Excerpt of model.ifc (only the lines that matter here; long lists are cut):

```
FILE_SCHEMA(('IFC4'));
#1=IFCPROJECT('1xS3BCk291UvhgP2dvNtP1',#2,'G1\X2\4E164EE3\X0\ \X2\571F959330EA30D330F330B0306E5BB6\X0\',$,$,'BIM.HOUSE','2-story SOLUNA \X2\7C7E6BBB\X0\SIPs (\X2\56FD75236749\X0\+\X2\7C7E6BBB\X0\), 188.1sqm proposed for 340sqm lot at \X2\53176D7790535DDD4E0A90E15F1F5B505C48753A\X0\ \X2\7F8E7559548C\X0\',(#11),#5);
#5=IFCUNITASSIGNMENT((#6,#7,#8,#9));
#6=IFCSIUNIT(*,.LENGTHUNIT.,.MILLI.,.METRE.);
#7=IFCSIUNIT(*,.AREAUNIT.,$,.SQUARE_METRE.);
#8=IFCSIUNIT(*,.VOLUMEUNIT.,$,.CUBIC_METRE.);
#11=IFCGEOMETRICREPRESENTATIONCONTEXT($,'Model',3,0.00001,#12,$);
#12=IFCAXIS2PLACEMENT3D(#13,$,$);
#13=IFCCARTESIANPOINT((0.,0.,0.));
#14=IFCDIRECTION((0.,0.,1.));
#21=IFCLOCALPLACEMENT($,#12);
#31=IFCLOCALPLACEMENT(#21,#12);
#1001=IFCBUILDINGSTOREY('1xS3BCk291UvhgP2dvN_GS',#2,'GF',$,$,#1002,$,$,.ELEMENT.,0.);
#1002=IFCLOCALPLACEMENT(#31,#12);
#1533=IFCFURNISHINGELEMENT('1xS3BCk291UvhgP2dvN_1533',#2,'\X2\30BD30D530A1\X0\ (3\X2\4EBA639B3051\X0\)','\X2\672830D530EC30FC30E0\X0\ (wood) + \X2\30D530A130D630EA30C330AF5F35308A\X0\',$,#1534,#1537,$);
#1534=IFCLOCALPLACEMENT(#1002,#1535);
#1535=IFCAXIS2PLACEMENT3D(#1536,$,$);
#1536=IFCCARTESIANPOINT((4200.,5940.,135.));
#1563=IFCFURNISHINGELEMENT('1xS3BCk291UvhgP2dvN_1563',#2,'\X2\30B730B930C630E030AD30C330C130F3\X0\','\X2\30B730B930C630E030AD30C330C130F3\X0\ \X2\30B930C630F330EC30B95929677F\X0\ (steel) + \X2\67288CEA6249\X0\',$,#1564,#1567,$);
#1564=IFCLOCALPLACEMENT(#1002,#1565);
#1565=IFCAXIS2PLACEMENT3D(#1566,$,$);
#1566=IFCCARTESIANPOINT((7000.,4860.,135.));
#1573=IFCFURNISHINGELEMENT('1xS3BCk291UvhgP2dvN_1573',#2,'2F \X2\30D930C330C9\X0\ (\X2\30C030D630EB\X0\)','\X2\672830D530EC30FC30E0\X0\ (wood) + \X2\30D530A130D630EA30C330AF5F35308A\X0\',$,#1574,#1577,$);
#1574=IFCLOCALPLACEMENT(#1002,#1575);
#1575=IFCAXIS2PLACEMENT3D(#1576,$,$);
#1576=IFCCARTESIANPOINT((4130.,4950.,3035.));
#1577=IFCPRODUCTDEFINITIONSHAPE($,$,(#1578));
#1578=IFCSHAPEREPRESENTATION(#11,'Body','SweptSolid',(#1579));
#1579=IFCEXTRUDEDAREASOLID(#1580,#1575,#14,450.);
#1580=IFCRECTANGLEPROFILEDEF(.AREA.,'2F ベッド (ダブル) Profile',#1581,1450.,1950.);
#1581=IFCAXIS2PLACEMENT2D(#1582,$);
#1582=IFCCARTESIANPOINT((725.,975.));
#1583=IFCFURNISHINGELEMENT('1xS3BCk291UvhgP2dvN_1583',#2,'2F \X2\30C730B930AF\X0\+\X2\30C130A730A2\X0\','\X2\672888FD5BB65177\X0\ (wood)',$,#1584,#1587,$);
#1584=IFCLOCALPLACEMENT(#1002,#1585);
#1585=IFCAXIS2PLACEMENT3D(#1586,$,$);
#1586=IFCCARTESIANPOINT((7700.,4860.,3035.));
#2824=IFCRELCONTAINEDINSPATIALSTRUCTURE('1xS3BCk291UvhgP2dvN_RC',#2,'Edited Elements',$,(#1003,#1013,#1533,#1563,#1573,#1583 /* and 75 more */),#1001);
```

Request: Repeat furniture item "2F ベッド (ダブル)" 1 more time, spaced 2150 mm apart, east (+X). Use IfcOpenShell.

```python
import numpy as np
import ifcopenshell
import ifcopenshell.api.geometry
import ifcopenshell.api.root
import ifcopenshell.util.element
import ifcopenshell.util.placement

model = ifcopenshell.open("model.ifc")


def reuse_history(source, copy):
    """copy_class also copies each property set's owner history, people and application; keep the originals."""
    for rel in copy.IsDefinedBy:
        if rel.is_a("IfcRelDefinesByProperties") and (history := rel.RelatingPropertyDefinition.OwnerHistory):
            rel.RelatingPropertyDefinition.OwnerHistory = source.OwnerHistory
            ifcopenshell.util.element.remove_deep2(model, history)


source = model.by_id(1573)
base = ifcopenshell.util.placement.get_local_placement(source.ObjectPlacement)
step = np.array([1.0, 0.0, 0.0]) * 2150.0

for i in range(1, 2):
    copy = ifcopenshell.api.root.copy_class(model, product=source)
    copy.Representation = ifcopenshell.util.element.copy_deep(
        model, source.Representation, exclude=["IfcGeometricRepresentationContext", "IfcRepresentationMap"]
    )
    reuse_history(source, copy)
    matrix = base.copy()
    matrix[:3, 3] += i * step
    print("added at", matrix[:3, 3].round(3) + 0.0)
    ifcopenshell.api.geometry.edit_object_placement(model, product=copy, matrix=matrix, is_si=False)

model.write("model_rev.ifc")
```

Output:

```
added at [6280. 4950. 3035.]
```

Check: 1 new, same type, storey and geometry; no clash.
